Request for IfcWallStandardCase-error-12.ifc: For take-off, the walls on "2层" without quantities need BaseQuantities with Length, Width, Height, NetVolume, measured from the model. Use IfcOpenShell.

First a look at what the model holds.

```python
import ifcopenshell
import ifcopenshell.util.element
import ifcopenshell.util.unit

model = ifcopenshell.open("IfcWallStandardCase-error-12.ifc")
print(model.schema)
for unit_type in ("LENGTHUNIT", "AREAUNIT", "VOLUMEUNIT"):
    print(unit_type, ifcopenshell.util.unit.calculate_unit_scale(model, unit_type))
storey = next(s for s in model.by_type("IfcBuildingStorey") if s.Name == "2层")
walls = [e for e in ifcopenshell.util.element.get_decomposition(storey) if e.is_a("IfcWall")]
for e in sorted(walls, key=lambda e: e.id()):
    print(e.id(), e.is_a(), e.Name, list(ifcopenshell.util.element.get_psets(e, qtos_only=True)), sep=" | ")
```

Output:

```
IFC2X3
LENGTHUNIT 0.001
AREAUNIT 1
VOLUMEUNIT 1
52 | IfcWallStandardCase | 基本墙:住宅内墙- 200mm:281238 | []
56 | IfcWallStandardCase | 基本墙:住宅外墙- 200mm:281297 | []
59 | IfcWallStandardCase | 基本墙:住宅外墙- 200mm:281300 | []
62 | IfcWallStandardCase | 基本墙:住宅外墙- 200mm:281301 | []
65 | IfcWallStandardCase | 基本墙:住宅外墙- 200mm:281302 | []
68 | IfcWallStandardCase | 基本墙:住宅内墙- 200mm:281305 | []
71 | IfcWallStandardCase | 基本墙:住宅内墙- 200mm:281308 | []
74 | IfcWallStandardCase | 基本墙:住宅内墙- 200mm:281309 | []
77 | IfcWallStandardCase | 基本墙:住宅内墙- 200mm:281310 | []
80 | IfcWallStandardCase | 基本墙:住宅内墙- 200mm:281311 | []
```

```python
import ifcopenshell
import ifcopenshell.api.pset
import ifcopenshell.geom
import ifcopenshell.util.element
import ifcopenshell.util.shape
import ifcopenshell.util.unit

model = ifcopenshell.open("IfcWallStandardCase-error-12.ifc")
unit_scale = ifcopenshell.util.unit.calculate_unit_scale(model)
volume_scale = ifcopenshell.util.unit.calculate_unit_scale(model, "VOLUMEUNIT")
settings = ifcopenshell.geom.settings()

storey = next(s for s in model.by_type("IfcBuildingStorey") if s.Name == "2层")
walls = [e for e in ifcopenshell.util.element.get_decomposition(storey) if e.is_a("IfcWall")]

for e in sorted(walls, key=lambda e: e.id()):
    if ifcopenshell.util.element.get_psets(e, qtos_only=True, should_inherit=False):
        continue
    # Geometry comes back in metres, in the element's own axes.
    shape = ifcopenshell.geom.create_shape(settings, e)
    values = {
        "Length": ifcopenshell.util.shape.get_x(shape.geometry) / unit_scale,
        "Width": ifcopenshell.util.shape.get_y(shape.geometry) / unit_scale,
        "Height": ifcopenshell.util.shape.get_z(shape.geometry) / unit_scale,
        "NetVolume": ifcopenshell.util.shape.get_volume(shape.geometry) / volume_scale,
    }
    qto = ifcopenshell.api.pset.add_qto(model, product=e, name="BaseQuantities")
    ifcopenshell.api.pset.edit_qto(model, qto=qto, properties=values)
    print(e.id(), {k: round(v, 3) for k, v in values.items()})

model.write("IfcWallStandardCase-error-12-out.ifc")
```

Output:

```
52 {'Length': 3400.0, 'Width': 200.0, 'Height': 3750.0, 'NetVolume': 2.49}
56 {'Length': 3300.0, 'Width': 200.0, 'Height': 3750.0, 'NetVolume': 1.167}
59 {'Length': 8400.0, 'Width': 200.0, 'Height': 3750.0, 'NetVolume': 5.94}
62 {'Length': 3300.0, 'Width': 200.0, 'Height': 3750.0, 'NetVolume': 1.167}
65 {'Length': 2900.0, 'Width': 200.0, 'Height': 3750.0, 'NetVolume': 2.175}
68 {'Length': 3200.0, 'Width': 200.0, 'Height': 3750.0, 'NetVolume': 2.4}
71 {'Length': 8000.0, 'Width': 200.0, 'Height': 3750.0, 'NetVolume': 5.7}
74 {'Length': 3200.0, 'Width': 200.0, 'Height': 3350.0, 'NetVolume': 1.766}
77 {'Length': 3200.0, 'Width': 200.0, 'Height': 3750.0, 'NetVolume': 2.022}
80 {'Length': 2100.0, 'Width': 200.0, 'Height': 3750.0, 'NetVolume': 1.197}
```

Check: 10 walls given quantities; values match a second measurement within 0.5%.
